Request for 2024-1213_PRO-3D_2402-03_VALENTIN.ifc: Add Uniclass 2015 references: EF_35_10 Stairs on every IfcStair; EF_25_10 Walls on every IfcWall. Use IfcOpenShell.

First a look at what the model holds.

```python
import ifcopenshell

model = ifcopenshell.open("2024-1213_PRO-3D_2402-03_VALENTIN.ifc")
print(model.schema)
print("classifications:", [c.Name for c in model.by_type("IfcClassification")])
for ifc_class in ("IfcDoor", "IfcRoof", "IfcStair", "IfcWall", "IfcWindow"):
    print(ifc_class, len(model.by_type(ifc_class)))
```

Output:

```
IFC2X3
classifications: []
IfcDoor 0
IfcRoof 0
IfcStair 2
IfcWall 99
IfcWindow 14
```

```python
import ifcopenshell
import ifcopenshell.api.classification

model = ifcopenshell.open("2024-1213_PRO-3D_2402-03_VALENTIN.ifc")

# IFC2X3 requires Source and Edition and has no link from the project to the system.
system = model.create_entity("IfcClassification", Source="NBS", Edition="2015", Name="Uniclass 2015")

codes = {
    "IfcStair": ("EF_35_10", "Stairs"),
    "IfcWall": ("EF_25_10", "Walls"),
}
for ifc_class, (code, name) in codes.items():
    products = model.by_type(ifc_class)
    ifcopenshell.api.classification.add_reference(
        model, products=products, classification=system, identification=code, name=name
    )
    print(code, len(products))

model.write("2024-1213_PRO-3D_2402-03_VALENTIN_rev.ifc")
```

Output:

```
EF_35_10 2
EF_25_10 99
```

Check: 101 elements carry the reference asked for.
